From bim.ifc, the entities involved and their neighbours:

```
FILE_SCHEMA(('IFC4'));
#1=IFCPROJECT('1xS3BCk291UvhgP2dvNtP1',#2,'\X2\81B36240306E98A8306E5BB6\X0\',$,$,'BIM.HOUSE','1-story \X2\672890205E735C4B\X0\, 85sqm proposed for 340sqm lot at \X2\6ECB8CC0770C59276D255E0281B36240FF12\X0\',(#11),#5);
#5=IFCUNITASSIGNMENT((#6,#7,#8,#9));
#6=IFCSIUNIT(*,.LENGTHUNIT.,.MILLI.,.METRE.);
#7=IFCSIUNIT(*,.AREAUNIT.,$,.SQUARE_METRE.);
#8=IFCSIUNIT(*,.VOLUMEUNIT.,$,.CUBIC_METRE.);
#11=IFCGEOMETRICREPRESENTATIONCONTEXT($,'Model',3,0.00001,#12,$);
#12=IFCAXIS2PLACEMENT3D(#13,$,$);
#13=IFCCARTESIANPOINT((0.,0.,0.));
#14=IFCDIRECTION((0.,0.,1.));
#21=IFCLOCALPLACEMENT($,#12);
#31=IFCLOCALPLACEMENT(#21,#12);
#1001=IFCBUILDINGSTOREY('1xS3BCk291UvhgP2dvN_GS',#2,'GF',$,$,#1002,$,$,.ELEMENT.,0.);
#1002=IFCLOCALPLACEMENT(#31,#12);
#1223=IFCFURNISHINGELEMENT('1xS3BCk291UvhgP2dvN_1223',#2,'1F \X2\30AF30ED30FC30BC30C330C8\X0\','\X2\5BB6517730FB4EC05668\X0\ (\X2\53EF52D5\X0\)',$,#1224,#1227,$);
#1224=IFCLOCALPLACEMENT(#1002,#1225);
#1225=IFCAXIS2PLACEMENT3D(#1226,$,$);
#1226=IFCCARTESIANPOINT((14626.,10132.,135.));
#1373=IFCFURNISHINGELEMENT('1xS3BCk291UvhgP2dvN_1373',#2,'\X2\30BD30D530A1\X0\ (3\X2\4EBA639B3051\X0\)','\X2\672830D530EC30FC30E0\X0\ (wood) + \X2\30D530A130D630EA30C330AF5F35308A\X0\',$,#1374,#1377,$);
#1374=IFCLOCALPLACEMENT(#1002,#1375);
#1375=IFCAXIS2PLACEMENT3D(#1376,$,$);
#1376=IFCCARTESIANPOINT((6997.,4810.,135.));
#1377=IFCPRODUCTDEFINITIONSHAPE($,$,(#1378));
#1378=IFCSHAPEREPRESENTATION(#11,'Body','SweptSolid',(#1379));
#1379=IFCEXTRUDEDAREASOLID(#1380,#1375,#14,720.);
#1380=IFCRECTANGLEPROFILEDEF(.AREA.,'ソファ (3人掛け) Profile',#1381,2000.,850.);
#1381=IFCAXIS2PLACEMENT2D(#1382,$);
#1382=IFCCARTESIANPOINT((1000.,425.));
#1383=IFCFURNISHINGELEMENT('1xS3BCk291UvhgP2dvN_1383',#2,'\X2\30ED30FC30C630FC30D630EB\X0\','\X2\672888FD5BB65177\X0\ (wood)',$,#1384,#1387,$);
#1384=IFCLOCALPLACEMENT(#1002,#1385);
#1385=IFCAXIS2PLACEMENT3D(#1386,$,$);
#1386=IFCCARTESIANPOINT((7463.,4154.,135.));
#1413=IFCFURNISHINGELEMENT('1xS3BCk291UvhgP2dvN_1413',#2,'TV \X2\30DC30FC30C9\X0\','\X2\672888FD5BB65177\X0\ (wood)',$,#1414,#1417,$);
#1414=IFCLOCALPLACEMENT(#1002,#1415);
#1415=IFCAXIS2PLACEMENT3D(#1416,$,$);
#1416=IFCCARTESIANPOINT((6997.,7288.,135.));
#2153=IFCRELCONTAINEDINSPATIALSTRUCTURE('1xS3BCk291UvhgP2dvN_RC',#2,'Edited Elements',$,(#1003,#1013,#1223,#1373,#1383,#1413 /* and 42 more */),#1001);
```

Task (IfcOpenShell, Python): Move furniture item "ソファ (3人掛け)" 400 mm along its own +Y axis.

```python
import ifcopenshell
import ifcopenshell.api.geometry
import ifcopenshell.util.placement
import ifcopenshell.util.unit

model = ifcopenshell.open("bim.ifc")
unit_scale = ifcopenshell.util.unit.calculate_unit_scale(model)

item = model.by_guid("1xS3BCk291UvhgP2dvN_1373")
matrix = ifcopenshell.util.placement.get_local_placement(item.ObjectPlacement)
matrix[:3, 3] += matrix[:3, 1] * 0.4 / unit_scale
ifcopenshell.api.geometry.edit_object_placement(model, product=item, matrix=matrix, is_si=False)

print(ifcopenshell.util.placement.get_local_placement(item.ObjectPlacement).round(3) + 0.0)

model.write("bim_rev.ifc")
```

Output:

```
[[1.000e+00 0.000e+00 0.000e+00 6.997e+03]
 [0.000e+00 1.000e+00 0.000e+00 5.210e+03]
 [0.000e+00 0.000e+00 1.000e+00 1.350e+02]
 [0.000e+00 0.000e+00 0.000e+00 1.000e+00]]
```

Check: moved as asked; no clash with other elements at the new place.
